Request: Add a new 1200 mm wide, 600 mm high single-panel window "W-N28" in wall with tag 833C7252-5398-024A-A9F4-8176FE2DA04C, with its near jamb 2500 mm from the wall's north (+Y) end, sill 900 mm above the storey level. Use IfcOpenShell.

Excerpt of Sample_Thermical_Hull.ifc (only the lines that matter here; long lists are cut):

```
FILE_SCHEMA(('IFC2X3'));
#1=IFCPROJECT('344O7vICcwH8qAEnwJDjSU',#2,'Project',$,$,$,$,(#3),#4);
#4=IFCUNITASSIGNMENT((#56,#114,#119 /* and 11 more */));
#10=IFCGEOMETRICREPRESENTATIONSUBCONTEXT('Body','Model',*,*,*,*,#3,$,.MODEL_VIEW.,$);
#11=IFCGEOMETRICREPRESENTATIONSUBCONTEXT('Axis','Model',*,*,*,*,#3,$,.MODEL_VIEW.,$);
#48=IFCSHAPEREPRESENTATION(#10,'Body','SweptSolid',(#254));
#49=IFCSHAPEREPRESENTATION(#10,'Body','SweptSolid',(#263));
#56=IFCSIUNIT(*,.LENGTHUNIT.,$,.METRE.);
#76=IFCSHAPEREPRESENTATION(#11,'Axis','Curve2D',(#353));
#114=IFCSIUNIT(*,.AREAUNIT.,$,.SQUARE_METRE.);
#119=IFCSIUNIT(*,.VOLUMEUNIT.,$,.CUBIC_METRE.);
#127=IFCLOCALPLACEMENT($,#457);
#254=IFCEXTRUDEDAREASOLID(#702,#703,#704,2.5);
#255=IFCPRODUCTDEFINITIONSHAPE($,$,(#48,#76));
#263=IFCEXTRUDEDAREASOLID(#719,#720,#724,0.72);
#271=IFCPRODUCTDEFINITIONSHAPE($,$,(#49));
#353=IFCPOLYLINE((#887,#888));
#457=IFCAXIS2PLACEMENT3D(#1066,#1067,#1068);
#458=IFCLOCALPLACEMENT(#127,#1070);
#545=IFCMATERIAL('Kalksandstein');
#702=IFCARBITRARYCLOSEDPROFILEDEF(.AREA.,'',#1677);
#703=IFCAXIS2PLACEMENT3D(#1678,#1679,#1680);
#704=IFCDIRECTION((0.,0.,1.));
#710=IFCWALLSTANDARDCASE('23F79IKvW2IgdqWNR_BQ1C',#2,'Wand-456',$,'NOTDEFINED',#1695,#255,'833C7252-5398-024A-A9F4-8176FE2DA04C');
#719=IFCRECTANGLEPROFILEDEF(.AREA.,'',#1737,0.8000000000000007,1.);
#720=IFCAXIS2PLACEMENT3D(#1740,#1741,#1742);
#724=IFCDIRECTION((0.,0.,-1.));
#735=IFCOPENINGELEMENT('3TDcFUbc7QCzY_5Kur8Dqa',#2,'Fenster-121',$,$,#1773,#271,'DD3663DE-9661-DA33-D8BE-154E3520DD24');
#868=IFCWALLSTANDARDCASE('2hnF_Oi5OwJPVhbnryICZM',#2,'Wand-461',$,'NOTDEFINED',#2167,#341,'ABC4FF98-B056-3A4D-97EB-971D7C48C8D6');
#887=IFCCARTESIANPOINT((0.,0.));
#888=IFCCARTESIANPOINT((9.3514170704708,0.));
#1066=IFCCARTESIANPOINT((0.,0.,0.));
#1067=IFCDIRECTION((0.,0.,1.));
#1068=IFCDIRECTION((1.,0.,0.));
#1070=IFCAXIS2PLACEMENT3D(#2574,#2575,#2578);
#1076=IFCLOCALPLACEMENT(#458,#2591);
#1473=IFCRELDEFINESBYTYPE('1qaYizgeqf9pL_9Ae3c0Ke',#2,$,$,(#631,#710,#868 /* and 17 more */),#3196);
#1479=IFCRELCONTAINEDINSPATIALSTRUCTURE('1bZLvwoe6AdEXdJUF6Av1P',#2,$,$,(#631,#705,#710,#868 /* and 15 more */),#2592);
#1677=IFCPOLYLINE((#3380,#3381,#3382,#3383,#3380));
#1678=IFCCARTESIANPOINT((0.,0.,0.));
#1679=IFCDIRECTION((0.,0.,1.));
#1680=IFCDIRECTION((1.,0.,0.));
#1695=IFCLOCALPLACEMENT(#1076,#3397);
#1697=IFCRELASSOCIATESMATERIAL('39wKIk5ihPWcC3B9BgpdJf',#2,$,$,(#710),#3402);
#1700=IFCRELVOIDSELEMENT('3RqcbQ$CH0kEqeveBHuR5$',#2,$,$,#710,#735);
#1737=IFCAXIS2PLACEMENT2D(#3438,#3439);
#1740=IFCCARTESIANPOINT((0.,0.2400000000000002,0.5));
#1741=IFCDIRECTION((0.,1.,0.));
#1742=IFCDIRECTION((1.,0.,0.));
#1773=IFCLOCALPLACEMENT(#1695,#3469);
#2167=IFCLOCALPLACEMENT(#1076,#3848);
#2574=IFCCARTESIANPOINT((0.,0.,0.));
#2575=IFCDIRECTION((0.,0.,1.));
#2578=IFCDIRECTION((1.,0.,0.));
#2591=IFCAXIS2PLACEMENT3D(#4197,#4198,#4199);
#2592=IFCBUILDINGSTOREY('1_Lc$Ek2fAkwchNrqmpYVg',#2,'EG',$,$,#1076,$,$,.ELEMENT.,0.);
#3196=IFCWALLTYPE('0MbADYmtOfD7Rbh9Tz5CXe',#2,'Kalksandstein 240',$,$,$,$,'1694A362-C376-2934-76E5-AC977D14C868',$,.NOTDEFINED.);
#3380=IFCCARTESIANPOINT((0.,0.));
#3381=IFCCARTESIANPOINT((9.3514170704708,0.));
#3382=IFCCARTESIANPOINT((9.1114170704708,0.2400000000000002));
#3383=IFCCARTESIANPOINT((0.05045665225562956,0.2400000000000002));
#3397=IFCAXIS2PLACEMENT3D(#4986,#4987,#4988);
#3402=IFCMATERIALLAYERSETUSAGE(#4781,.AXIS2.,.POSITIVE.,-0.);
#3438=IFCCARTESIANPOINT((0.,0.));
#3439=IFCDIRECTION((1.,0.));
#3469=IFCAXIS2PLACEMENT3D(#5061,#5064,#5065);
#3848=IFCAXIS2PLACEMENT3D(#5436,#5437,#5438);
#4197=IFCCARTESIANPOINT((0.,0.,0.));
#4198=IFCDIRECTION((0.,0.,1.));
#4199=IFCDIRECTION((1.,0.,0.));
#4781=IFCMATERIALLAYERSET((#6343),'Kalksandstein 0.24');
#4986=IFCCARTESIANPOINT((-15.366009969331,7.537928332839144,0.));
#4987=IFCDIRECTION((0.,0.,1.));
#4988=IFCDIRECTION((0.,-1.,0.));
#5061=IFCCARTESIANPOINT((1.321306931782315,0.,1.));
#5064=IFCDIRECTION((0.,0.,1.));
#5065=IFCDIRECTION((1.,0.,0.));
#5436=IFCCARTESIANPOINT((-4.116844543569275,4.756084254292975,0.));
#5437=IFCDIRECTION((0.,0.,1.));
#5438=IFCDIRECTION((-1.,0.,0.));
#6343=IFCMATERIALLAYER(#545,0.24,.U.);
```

```python
import numpy as np
import ifcopenshell
import ifcopenshell.api.feature
import ifcopenshell.api.geometry
import ifcopenshell.api.root
import ifcopenshell.api.spatial
import ifcopenshell.api.type
import ifcopenshell.geom
import ifcopenshell.util.element
import ifcopenshell.util.placement
import ifcopenshell.util.representation
import ifcopenshell.util.shape
import ifcopenshell.util.unit

model = ifcopenshell.open("Sample_Thermical_Hull.ifc")
unit_scale = ifcopenshell.util.unit.calculate_unit_scale(model)
settings = ifcopenshell.geom.settings()


def volume(element):
    """Net volume in cubic metres, openings subtracted."""
    shape = ifcopenshell.geom.create_shape(settings, element)
    return ifcopenshell.util.shape.get_volume(shape.geometry)


wall = model.by_guid("23F79IKvW2IgdqWNR_BQ1C")
storey = ifcopenshell.util.element.get_container(wall, ifc_class="IfcBuildingStorey")
context = ifcopenshell.util.representation.get_context(model, "Model", "Body", "MODEL_VIEW")
before = volume(wall)

width, height, from_end, sill = 1.2, 0.6, 2.5, 0.9  # metres

# The wall runs along its own X axis, and the end named is its -X end.
wall_shape = ifcopenshell.geom.create_shape(settings, wall)
x, y, z = ifcopenshell.util.shape.get_vertices(wall_shape.geometry).T
start = x.min() + from_end
face, thickness = float(y.min()), float(y.max() - y.min())
wall_matrix = ifcopenshell.util.placement.get_local_placement(wall.ObjectPlacement)
level = ifcopenshell.util.placement.get_local_placement(storey.ObjectPlacement)[2, 3]


def in_wall(x, y):
    """Placement at x, y metres in the wall's axes, at sill height."""
    matrix = wall_matrix.copy()
    matrix[:, 3] = wall_matrix @ np.array([x / unit_scale, y / unit_scale, 0.0, 1.0])
    matrix[2, 3] = level + sill / unit_scale
    return matrix


# Opening: a box that overshoots both wall faces by 50 mm.
opening = ifcopenshell.api.root.create_entity(model, ifc_class="IfcOpeningElement")
box = ifcopenshell.api.geometry.add_wall_representation(
    model, context=context, length=width, height=height, thickness=thickness + 0.1
)
ifcopenshell.api.geometry.assign_representation(model, product=opening, representation=box)
ifcopenshell.api.geometry.edit_object_placement(model, product=opening, matrix=in_wall(start, face - 0.05), is_si=False)
ifcopenshell.api.feature.add_feature(model, feature=opening, element=wall)

window = ifcopenshell.api.root.create_entity(model, ifc_class="IfcWindow", name="W-N28")
window.OverallWidth, window.OverallHeight = width / unit_scale, height / unit_scale
body = ifcopenshell.api.geometry.add_window_representation(
    model,
    context=context,
    overall_width=window.OverallWidth,
    overall_height=window.OverallHeight,
    partition_type="SINGLE_PANEL",
)
ifcopenshell.api.geometry.assign_representation(model, product=window, representation=body)
ifcopenshell.api.spatial.assign_container(model, products=[window], relating_structure=storey)
fills = ifcopenshell.api.feature.add_filling(model, opening=opening, element=window)
fills.OwnerHistory = window.OwnerHistory  # required in IFC2X3

# IFC2X3 keeps the operation on the window style.
style = ifcopenshell.api.root.create_entity(model, ifc_class="IfcWindowStyle", name="W-N28")
style.OperationType, style.ConstructionType = "SINGLE_PANEL", "NOTDEFINED"
style.ParameterTakesPrecedence = style.Sizeable = False
ifcopenshell.api.type.assign_type(model, related_objects=[window], relating_type=style)

# Centre the window in the wall's thickness.
ifcopenshell.api.geometry.edit_object_placement(model, product=window, matrix=in_wall(start, face), is_si=False)
window_shape = ifcopenshell.geom.create_shape(settings, window)
depth = ifcopenshell.util.shape.get_vertices(window_shape.geometry)[:, 1]
offset = face + thickness / 2 - (depth.min() + depth.max()) / 2
ifcopenshell.api.geometry.edit_object_placement(model, product=window, matrix=in_wall(start, offset), is_si=False)

after = volume(wall)

print(f"wall volume {before:.3f} -> {after:.3f} m3")

model.write("Sample_Thermical_Hull_rev.ifc")
```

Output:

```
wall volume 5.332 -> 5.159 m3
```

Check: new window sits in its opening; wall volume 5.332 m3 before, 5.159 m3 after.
